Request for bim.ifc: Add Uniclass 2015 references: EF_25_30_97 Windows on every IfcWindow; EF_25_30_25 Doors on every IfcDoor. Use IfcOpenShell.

First a look at what the model holds.

```python
import ifcopenshell

model = ifcopenshell.open("bim.ifc")
print(model.schema)
print("classifications:", [c.Name for c in model.by_type("IfcClassification")])
for ifc_class in ("IfcDoor", "IfcRoof", "IfcStair", "IfcWall", "IfcWindow"):
    print(ifc_class, len(model.by_type(ifc_class)))
```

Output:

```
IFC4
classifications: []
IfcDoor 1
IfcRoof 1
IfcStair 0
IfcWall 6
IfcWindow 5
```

```python
import ifcopenshell
import ifcopenshell.api.classification

model = ifcopenshell.open("bim.ifc")

system = ifcopenshell.api.classification.add_classification(model, classification="Uniclass 2015")

codes = {
    "IfcWindow": ("EF_25_30_97", "Windows"),
    "IfcDoor": ("EF_25_30_25", "Doors"),
}
for ifc_class, (code, name) in codes.items():
    products = model.by_type(ifc_class)
    ifcopenshell.api.classification.add_reference(
        model, products=products, classification=system, identification=code, name=name
    )
    print(code, len(products))

model.write("bim_edited.ifc")
```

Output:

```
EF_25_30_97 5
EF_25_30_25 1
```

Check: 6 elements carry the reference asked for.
